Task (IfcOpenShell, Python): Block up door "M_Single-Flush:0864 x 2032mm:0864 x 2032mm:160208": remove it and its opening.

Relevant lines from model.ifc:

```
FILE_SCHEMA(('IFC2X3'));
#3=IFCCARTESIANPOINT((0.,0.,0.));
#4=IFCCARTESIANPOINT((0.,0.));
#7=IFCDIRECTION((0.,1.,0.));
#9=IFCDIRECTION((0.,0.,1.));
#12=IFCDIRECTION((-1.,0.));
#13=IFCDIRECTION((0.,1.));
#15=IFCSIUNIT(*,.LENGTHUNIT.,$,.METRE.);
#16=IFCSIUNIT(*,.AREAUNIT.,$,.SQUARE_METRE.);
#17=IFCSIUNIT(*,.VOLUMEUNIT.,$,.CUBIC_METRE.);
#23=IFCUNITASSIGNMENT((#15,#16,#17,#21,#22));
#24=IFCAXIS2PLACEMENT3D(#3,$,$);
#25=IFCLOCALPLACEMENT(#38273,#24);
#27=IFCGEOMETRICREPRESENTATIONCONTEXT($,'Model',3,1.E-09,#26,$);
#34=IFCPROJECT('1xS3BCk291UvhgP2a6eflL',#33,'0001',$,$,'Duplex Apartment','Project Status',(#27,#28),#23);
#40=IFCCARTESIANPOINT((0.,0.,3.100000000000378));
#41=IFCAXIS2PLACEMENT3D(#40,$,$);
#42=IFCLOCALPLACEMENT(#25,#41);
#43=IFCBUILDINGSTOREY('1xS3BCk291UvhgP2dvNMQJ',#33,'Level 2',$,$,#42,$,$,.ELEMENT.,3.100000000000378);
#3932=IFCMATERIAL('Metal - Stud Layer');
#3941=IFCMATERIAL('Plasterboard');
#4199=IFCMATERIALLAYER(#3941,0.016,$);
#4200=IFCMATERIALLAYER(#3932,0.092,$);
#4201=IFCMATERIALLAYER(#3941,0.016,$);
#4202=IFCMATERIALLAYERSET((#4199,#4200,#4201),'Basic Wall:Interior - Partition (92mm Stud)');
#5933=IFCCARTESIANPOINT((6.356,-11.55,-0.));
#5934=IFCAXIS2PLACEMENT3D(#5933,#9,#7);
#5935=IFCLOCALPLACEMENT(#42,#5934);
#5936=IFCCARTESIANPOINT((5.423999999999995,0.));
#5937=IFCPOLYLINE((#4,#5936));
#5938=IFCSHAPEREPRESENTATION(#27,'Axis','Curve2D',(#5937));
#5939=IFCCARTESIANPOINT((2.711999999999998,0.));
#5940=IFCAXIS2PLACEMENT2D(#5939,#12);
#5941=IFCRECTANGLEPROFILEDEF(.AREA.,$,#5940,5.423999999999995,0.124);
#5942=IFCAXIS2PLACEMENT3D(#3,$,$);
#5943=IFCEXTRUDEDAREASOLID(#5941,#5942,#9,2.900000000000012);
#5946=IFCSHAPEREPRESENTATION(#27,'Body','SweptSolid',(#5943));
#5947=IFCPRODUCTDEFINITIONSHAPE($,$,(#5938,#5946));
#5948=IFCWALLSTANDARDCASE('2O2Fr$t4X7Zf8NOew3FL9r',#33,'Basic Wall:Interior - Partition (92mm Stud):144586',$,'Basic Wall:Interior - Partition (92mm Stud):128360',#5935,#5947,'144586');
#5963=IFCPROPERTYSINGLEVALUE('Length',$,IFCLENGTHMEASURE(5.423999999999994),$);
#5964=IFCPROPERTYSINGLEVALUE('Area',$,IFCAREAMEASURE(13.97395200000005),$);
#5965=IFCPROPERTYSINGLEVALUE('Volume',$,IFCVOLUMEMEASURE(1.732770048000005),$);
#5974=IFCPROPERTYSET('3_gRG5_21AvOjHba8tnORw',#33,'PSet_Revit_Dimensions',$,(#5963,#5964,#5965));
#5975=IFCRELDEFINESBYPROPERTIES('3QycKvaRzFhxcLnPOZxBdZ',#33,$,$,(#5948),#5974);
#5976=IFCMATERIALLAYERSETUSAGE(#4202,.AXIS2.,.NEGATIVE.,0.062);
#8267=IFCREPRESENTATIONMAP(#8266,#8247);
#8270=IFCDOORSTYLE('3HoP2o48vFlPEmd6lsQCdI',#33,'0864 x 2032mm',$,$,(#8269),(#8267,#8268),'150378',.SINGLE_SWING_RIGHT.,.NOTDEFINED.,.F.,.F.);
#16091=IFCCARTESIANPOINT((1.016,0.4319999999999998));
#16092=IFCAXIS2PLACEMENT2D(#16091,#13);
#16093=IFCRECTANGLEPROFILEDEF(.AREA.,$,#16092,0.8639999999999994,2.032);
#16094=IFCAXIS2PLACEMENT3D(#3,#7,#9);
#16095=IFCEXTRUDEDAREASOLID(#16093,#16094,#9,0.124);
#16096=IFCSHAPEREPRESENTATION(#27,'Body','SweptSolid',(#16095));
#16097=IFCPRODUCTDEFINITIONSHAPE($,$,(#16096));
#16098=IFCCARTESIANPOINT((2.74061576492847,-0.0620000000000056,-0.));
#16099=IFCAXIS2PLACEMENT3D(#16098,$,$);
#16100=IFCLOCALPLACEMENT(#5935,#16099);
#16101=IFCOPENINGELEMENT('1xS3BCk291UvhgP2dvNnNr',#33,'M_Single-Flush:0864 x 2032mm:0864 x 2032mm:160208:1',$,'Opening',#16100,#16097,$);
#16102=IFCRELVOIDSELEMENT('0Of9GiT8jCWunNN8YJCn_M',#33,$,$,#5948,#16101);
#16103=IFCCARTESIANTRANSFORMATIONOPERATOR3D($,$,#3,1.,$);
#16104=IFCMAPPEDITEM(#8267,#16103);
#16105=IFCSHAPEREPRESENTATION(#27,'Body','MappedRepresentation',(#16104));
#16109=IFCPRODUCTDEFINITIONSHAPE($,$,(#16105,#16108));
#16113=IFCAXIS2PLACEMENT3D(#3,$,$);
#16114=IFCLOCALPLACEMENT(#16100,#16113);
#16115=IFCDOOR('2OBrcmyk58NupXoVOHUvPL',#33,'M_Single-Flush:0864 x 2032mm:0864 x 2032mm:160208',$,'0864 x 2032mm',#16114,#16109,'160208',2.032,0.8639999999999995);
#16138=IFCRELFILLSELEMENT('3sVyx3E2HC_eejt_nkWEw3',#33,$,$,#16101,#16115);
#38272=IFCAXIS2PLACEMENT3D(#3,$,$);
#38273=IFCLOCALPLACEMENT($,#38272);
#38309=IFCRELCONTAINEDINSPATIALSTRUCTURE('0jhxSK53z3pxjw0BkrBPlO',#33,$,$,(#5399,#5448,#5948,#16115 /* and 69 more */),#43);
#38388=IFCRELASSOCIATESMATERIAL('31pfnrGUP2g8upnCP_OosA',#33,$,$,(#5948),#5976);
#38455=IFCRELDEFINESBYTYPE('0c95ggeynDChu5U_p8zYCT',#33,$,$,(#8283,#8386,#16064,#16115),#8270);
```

```python
import ifcopenshell
import ifcopenshell.api.feature
import ifcopenshell.api.pset
import ifcopenshell.api.root
import ifcopenshell.geom
import ifcopenshell.util.element
import ifcopenshell.util.shape
import ifcopenshell.util.unit

model = ifcopenshell.open("model.ifc")
area_scale = ifcopenshell.util.unit.calculate_unit_scale(model, "AREAUNIT")
volume_scale = ifcopenshell.util.unit.calculate_unit_scale(model, "VOLUMEUNIT")
settings = ifcopenshell.geom.settings()


def volume(element):
    """Net volume in cubic metres, openings subtracted."""
    shape = ifcopenshell.geom.create_shape(settings, element)
    return ifcopenshell.util.shape.get_volume(shape.geometry)


door = model.by_guid("2OBrcmyk58NupXoVOHUvPL")
opening = door.FillsVoids[0].RelatingOpeningElement
wall = opening.VoidsElements[0].RelatingBuildingElement
before = volume(wall)

ifcopenshell.api.root.remove_product(model, product=door)
ifcopenshell.api.feature.remove_feature(model, feature=opening)

after = volume(wall)
thickness = 0.124  # wall thickness in metres

# Update the wall's stored quantities.
pset = model.by_id(ifcopenshell.util.element.get_pset(wall, "PSet_Revit_Dimensions", should_inherit=False)["id"])
ifcopenshell.api.pset.edit_pset(model, pset=pset, properties={
    "Area": model.create_entity("IfcAreaMeasure", after / thickness / area_scale),
    "Volume": model.create_entity("IfcVolumeMeasure", after / volume_scale),
})

print(f"wall volume {before:.3f} -> {after:.3f} m3")

model.write("model_edited.ifc")
```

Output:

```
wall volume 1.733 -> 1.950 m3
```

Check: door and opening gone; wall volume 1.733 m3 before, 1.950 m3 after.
